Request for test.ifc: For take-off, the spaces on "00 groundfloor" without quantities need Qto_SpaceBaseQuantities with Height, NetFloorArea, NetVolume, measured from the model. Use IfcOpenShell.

First a look at what the model holds.

```python
import ifcopenshell
import ifcopenshell.util.element
import ifcopenshell.util.unit

model = ifcopenshell.open("test.ifc")
print(model.schema)
for unit_type in ("LENGTHUNIT", "AREAUNIT", "VOLUMEUNIT"):
    print(unit_type, ifcopenshell.util.unit.calculate_unit_scale(model, unit_type))
storey = next(s for s in model.by_type("IfcBuildingStorey") if s.Name == "00 groundfloor")
spaces = [e for e in ifcopenshell.util.element.get_decomposition(storey) if e.is_a("IfcSpace")]
for e in sorted(spaces, key=lambda e: e.id()):
    print(e.id(), e.is_a(), e.Name, list(ifcopenshell.util.element.get_psets(e, qtos_only=True)), sep=" | ")
```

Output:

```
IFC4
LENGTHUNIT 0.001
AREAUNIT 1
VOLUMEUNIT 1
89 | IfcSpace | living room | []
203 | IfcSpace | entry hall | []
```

```python
import ifcopenshell
import ifcopenshell.api.pset
import ifcopenshell.geom
import ifcopenshell.util.element
import ifcopenshell.util.shape
import ifcopenshell.util.unit

model = ifcopenshell.open("test.ifc")
unit_scale = ifcopenshell.util.unit.calculate_unit_scale(model)
area_scale = ifcopenshell.util.unit.calculate_unit_scale(model, "AREAUNIT")
volume_scale = ifcopenshell.util.unit.calculate_unit_scale(model, "VOLUMEUNIT")
settings = ifcopenshell.geom.settings()

storey = next(s for s in model.by_type("IfcBuildingStorey") if s.Name == "00 groundfloor")
spaces = [e for e in ifcopenshell.util.element.get_decomposition(storey) if e.is_a("IfcSpace")]

for e in sorted(spaces, key=lambda e: e.id()):
    if ifcopenshell.util.element.get_psets(e, qtos_only=True, should_inherit=False):
        continue
    # Geometry comes back in metres, in the element's own axes.
    shape = ifcopenshell.geom.create_shape(settings, e)
    values = {
        "Height": ifcopenshell.util.shape.get_z(shape.geometry) / unit_scale,
        "NetFloorArea": ifcopenshell.util.shape.get_footprint_area(shape.geometry) / area_scale,
        "NetVolume": ifcopenshell.util.shape.get_volume(shape.geometry) / volume_scale,
    }
    qto = ifcopenshell.api.pset.add_qto(model, product=e, name="Qto_SpaceBaseQuantities")
    ifcopenshell.api.pset.edit_qto(model, qto=qto, properties=values)
    print(e.id(), {k: round(v, 3) for k, v in values.items()})

model.write("test-out.ifc")
```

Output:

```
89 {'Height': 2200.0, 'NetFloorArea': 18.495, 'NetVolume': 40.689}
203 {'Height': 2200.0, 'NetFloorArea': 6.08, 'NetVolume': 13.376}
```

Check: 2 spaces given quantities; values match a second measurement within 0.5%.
